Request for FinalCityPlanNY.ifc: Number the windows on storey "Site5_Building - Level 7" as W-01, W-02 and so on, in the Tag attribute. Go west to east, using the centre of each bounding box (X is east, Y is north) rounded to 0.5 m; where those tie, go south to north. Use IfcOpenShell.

First a look at what the model holds.

```python
import ifcopenshell
import ifcopenshell.util.element
import ifcopenshell.util.placement

model = ifcopenshell.open("FinalCityPlanNY.ifc")
print(model.schema)
storey = next(s for s in model.by_type("IfcBuildingStorey") if s.Name == "Site5_Building - Level 7")
windows = [e for e in ifcopenshell.util.element.get_decomposition(storey) if e.is_a("IfcWindow")]
for e in sorted(windows, key=lambda e: e.id()):
    origin = ifcopenshell.util.placement.get_local_placement(e.ObjectPlacement)[:3, 3]
    print(e.id(), e.Tag, e.Name, origin.round(2) + 0.0, sep=" | ")
```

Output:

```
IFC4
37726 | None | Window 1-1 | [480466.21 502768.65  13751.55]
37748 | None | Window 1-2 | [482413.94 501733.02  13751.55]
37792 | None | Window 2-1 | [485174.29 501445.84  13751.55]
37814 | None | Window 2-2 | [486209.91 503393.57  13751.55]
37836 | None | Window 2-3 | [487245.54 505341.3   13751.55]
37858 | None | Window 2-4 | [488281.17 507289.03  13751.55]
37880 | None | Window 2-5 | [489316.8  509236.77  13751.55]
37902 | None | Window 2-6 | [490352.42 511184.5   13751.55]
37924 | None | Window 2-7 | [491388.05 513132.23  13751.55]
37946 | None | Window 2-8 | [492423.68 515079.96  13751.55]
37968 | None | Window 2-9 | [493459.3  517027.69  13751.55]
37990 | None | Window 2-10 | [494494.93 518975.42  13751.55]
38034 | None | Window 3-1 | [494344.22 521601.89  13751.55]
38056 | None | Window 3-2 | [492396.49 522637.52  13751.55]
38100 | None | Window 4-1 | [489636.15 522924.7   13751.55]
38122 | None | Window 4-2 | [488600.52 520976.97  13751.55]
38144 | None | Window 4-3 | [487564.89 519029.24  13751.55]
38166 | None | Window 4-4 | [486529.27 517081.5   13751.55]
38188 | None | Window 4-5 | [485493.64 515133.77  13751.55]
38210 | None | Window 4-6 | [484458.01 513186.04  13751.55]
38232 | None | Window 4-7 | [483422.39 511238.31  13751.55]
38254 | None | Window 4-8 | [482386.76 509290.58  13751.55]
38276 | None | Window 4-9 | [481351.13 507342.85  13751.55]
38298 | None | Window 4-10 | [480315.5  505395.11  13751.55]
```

```python
import ifcopenshell
import ifcopenshell.geom
import ifcopenshell.util.element
import ifcopenshell.util.shape

model = ifcopenshell.open("FinalCityPlanNY.ifc")
settings = ifcopenshell.geom.settings()
settings.set("use-world-coords", True)


def centre(element):
    shape = ifcopenshell.geom.create_shape(settings, element)
    return ifcopenshell.util.shape.get_bbox_centroid(shape.geometry)


storey = next(s for s in model.by_type("IfcBuildingStorey") if s.Name == "Site5_Building - Level 7")
windows = [e for e in ifcopenshell.util.element.get_decomposition(storey) if e.is_a("IfcWindow")]

# Insertion points can sit at a corner or the storey origin, so sort by the geometry (in metres).
centres = {e: centre(e) for e in windows}
windows.sort(key=lambda e: (round(centres[e][0] / 0.5), centres[e][1]))

for i, e in enumerate(windows, start=1):
    number = f"W-{i:02d}"
    e.Tag = number
    print(e.id(), number)

model.write("FinalCityPlanNY_updated.ifc")
```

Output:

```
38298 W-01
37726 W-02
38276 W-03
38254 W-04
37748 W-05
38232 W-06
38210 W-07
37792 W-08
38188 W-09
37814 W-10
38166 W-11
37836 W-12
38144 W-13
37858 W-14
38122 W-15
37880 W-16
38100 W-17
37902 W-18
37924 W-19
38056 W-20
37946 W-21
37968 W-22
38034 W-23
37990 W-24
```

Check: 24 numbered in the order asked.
